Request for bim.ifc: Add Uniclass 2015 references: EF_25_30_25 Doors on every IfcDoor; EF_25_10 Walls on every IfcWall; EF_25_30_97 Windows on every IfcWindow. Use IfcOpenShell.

First a look at what the model holds.

```python
import ifcopenshell

model = ifcopenshell.open("bim.ifc")
print(model.schema)
print("classifications:", [c.Name for c in model.by_type("IfcClassification")])
for ifc_class in ("IfcDoor", "IfcRoof", "IfcStair", "IfcWall", "IfcWindow"):
    print(ifc_class, len(model.by_type(ifc_class)))
```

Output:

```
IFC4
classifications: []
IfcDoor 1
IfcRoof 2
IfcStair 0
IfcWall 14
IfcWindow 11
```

```python
import ifcopenshell
import ifcopenshell.api.classification

model = ifcopenshell.open("bim.ifc")

system = ifcopenshell.api.classification.add_classification(model, classification="Uniclass 2015")

codes = {
    "IfcDoor": ("EF_25_30_25", "Doors"),
    "IfcWall": ("EF_25_10", "Walls"),
    "IfcWindow": ("EF_25_30_97", "Windows"),
}
for ifc_class, (code, name) in codes.items():
    products = model.by_type(ifc_class)
    ifcopenshell.api.classification.add_reference(
        model, products=products, classification=system, identification=code, name=name
    )
    print(code, len(products))

model.write("bim-out.ifc")
```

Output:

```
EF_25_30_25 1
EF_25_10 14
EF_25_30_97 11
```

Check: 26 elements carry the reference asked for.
